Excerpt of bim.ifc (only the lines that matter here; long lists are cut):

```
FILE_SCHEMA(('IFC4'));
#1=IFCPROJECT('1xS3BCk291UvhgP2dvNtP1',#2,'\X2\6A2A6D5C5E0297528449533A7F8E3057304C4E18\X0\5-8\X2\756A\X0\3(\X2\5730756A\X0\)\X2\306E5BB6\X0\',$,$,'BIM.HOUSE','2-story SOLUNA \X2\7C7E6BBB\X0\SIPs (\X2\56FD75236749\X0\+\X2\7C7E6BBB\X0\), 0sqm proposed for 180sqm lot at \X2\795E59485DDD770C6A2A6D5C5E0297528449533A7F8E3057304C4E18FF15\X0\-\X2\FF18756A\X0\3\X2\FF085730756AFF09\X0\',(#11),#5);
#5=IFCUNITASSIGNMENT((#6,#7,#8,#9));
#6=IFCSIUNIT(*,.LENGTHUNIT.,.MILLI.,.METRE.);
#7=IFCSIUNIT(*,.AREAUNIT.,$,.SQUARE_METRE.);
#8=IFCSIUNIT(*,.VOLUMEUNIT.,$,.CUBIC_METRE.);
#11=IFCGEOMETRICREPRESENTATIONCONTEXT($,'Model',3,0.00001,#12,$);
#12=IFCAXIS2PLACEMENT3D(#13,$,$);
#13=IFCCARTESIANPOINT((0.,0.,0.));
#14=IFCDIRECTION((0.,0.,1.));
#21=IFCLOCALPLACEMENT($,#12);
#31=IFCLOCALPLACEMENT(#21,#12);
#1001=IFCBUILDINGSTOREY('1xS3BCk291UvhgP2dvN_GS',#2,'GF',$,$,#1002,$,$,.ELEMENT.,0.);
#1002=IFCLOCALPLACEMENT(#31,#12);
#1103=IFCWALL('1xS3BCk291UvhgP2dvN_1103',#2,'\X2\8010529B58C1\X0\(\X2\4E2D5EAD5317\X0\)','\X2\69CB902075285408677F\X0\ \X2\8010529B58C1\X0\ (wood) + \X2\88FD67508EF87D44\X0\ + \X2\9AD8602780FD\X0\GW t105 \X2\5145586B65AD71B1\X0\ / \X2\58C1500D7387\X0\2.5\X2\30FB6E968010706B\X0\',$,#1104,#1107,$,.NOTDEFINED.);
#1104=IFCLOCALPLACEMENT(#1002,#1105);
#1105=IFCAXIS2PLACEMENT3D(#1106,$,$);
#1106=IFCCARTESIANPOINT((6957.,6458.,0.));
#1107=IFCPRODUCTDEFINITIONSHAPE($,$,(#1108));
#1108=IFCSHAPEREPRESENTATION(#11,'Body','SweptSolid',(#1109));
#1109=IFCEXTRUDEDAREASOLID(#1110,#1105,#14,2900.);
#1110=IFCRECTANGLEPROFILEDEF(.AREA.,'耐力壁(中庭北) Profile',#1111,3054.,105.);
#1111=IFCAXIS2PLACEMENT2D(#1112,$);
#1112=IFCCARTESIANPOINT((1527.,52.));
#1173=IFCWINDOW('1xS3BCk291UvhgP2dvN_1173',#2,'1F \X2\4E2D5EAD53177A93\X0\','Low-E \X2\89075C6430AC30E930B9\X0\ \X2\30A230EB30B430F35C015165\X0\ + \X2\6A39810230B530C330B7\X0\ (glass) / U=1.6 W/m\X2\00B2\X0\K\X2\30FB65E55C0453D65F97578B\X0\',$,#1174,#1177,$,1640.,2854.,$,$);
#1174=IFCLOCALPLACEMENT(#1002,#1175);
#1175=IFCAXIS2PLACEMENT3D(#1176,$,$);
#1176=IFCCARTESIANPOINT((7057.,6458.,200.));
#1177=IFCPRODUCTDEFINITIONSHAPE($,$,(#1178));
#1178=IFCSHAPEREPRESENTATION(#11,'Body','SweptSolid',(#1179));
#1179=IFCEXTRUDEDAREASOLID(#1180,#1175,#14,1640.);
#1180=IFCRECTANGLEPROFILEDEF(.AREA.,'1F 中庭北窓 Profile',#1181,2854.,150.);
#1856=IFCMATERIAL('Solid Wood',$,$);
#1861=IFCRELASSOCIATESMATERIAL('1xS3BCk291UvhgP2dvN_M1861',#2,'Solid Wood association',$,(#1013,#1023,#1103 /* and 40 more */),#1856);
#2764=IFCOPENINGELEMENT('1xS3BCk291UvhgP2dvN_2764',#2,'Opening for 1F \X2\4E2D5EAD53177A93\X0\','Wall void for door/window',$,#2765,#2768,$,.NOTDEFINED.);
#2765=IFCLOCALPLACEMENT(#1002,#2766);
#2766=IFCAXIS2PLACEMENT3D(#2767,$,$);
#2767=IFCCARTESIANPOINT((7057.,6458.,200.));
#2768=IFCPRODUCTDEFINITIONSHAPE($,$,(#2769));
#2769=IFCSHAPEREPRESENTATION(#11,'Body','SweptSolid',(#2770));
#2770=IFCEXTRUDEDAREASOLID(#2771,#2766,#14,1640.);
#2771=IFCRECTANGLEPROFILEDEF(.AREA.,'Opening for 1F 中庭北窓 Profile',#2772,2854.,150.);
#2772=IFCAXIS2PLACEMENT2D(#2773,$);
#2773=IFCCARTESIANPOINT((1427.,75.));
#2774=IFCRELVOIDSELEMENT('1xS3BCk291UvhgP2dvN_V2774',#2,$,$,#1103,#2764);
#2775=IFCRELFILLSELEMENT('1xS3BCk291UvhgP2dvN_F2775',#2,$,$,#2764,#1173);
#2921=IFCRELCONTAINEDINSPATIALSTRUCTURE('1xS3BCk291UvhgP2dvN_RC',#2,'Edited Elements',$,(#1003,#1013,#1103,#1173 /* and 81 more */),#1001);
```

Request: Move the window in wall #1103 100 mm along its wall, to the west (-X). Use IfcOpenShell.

```python
import ifcopenshell
import ifcopenshell.api.geometry
import ifcopenshell.util.placement
import ifcopenshell.util.unit

model = ifcopenshell.open("bim.ifc")
unit_scale = ifcopenshell.util.unit.calculate_unit_scale(model)

window = model.by_id(1173)
opening = window.FillsVoids[0].RelatingOpeningElement
wall = opening.VoidsElements[0].RelatingBuildingElement

wall_matrix = ifcopenshell.util.placement.get_local_placement(wall.ObjectPlacement)
shift = wall_matrix[:3, 0] * -0.1 / unit_scale
before = ifcopenshell.util.placement.get_local_placement(window.ObjectPlacement)[:3, 3].copy()

# The window is not placed relative to its opening, so move both.
for product in (opening, window):
    matrix = ifcopenshell.util.placement.get_local_placement(product.ObjectPlacement)
    matrix[:3, 3] += shift
    ifcopenshell.api.geometry.edit_object_placement(model, product=product, matrix=matrix, is_si=False)

after = ifcopenshell.util.placement.get_local_placement(window.ObjectPlacement)[:3, 3]
print("window moved by", (after - before).round(3) + 0.0)

model.write("bim_edited.ifc")
```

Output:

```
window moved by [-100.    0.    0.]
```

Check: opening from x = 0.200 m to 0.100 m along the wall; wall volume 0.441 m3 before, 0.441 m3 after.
